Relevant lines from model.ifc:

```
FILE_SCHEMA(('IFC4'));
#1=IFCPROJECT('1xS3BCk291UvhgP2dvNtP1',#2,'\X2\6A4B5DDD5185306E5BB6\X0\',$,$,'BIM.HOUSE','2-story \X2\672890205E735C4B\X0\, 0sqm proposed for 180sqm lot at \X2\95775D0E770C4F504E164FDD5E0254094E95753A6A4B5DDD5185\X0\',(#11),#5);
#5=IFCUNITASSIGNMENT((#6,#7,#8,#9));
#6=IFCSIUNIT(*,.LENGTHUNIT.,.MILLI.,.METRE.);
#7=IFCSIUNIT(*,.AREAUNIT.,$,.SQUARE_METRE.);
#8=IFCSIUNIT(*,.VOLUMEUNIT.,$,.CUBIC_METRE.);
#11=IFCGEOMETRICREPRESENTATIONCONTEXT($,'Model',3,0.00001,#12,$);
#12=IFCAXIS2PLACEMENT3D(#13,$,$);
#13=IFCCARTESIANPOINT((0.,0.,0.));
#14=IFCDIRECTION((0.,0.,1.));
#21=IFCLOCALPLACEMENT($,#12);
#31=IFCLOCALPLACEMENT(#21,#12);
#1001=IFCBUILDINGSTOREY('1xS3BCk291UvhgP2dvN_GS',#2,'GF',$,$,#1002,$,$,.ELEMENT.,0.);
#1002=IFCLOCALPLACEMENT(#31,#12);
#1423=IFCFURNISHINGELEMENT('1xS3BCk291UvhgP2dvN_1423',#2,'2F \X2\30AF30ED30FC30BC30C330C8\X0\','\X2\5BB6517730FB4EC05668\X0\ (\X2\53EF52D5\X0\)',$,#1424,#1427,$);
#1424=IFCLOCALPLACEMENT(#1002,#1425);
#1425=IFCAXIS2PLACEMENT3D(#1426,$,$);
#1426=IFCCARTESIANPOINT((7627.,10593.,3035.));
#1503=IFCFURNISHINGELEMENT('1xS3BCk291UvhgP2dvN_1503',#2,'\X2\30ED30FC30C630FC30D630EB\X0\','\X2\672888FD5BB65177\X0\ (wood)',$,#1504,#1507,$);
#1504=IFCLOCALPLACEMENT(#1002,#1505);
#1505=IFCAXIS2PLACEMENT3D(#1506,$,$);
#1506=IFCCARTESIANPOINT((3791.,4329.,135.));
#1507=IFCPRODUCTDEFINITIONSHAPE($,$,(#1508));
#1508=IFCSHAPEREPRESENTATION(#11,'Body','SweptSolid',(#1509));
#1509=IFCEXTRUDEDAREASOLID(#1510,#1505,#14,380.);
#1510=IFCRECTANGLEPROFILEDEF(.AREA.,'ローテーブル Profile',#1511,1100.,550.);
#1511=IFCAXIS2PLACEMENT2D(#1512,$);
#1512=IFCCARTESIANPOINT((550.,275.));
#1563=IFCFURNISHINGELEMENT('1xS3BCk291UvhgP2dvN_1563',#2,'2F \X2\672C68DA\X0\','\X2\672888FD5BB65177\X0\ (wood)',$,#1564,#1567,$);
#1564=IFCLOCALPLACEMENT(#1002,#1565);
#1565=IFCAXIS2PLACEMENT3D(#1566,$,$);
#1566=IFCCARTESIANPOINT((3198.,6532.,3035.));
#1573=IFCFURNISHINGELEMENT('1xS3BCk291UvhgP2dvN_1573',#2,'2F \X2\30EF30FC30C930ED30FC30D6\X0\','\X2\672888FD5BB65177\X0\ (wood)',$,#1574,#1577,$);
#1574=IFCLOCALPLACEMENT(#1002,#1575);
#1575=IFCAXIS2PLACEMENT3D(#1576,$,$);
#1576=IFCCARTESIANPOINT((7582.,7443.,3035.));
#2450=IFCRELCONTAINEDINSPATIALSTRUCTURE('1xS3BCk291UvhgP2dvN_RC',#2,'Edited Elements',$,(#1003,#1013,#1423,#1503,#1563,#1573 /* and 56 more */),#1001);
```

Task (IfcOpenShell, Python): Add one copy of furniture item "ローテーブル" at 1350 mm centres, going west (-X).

```python
import numpy as np
import ifcopenshell
import ifcopenshell.api.geometry
import ifcopenshell.api.root
import ifcopenshell.util.element
import ifcopenshell.util.placement
import ifcopenshell.util.unit

model = ifcopenshell.open("model.ifc")
unit_scale = ifcopenshell.util.unit.calculate_unit_scale(model)


def reuse_history(source, copy):
    """copy_class also copies each property set's owner history, people and application; keep the originals."""
    for rel in copy.IsDefinedBy:
        if rel.is_a("IfcRelDefinesByProperties") and (history := rel.RelatingPropertyDefinition.OwnerHistory):
            rel.RelatingPropertyDefinition.OwnerHistory = source.OwnerHistory
            ifcopenshell.util.element.remove_deep2(model, history)


source = model.by_id(1503)
base = ifcopenshell.util.placement.get_local_placement(source.ObjectPlacement)
step = np.array([-1.0, 0.0, 0.0]) * 1.35 / unit_scale

for i in range(1, 2):
    copy = ifcopenshell.api.root.copy_class(model, product=source)
    copy.Representation = ifcopenshell.util.element.copy_deep(
        model, source.Representation, exclude=["IfcGeometricRepresentationContext", "IfcRepresentationMap"]
    )
    reuse_history(source, copy)
    matrix = base.copy()
    matrix[:3, 3] += i * step
    print("added at", matrix[:3, 3].round(3) + 0.0)
    ifcopenshell.api.geometry.edit_object_placement(model, product=copy, matrix=matrix, is_si=False)

model.write("model_v2.ifc")
```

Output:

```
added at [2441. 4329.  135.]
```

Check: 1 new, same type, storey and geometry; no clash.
